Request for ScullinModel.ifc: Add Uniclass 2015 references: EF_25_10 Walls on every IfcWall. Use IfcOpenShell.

First a look at what the model holds.

```python
import ifcopenshell

model = ifcopenshell.open("ScullinModel.ifc")
print(model.schema)
print("classifications:", [c.Name for c in model.by_type("IfcClassification")])
for ifc_class in ("IfcDoor", "IfcRoof", "IfcStair", "IfcWall", "IfcWindow"):
    print(ifc_class, len(model.by_type(ifc_class)))
```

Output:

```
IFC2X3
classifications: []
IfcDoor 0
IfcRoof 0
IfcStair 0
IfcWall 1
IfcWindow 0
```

```python
import ifcopenshell
import ifcopenshell.api.classification

model = ifcopenshell.open("ScullinModel.ifc")

# IFC2X3 requires Source and Edition and has no link from the project to the system.
system = model.create_entity("IfcClassification", Source="NBS", Edition="2015", Name="Uniclass 2015")

codes = {
    "IfcWall": ("EF_25_10", "Walls"),
}
for ifc_class, (code, name) in codes.items():
    products = model.by_type(ifc_class)
    ifcopenshell.api.classification.add_reference(
        model, products=products, classification=system, identification=code, name=name
    )
    print(code, len(products))

model.write("ScullinModel_rev.ifc")
```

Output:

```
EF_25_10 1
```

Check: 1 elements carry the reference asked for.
